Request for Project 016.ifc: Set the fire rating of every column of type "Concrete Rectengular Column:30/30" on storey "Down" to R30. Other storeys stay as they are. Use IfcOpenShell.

First a look at what the model holds.

```python
import ifcopenshell
import ifcopenshell.util.element

model = ifcopenshell.open("Project 016.ifc")
print(model.schema)
storey = next(s for s in model.by_type("IfcBuildingStorey") if s.Name == "Down")
columns = [e for e in ifcopenshell.util.element.get_decomposition(storey) if e.is_a("IfcColumn")]
seen = {}
for e in columns:
    element_type = ifcopenshell.util.element.get_type(e)
    key = (element_type.Name if element_type != e and element_type else None, ifcopenshell.util.element.get_pset(e, "Pset_ColumnCommon", "FireRating"))
    seen[key] = seen.get(key, 0) + 1
for (name, value), count in sorted(seen.items(), key=str):
    print(count, "x", name, "|", value)
```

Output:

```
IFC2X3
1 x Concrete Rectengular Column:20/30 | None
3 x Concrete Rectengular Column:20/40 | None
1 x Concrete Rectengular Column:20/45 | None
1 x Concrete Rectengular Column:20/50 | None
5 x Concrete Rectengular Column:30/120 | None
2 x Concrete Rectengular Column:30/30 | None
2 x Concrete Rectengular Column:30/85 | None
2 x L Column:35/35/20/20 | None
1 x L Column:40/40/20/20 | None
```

```python
import ifcopenshell
import ifcopenshell.api.pset
import ifcopenshell.util.element

model = ifcopenshell.open("Project 016.ifc")

storey = next(s for s in model.by_type("IfcBuildingStorey") if s.Name == "Down")
columns = [e for e in ifcopenshell.util.element.get_decomposition(storey) if e.is_a("IfcColumn")]

count = 0
for e in columns:
    element_type = ifcopenshell.util.element.get_type(e)
    if element_type in (None, e) or element_type.Name != "Concrete Rectengular Column:30/30":
        continue
    # add_pset returns the element's existing set when there is one.
    pset = ifcopenshell.api.pset.add_pset(model, product=e, name="Pset_ColumnCommon")
    ifcopenshell.api.pset.edit_pset(model, pset=pset, properties={"FireRating": "R30"})
    count += 1

print(count, "columns updated")

model.write("Project 016-out.ifc")
```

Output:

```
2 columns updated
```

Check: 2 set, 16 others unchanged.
